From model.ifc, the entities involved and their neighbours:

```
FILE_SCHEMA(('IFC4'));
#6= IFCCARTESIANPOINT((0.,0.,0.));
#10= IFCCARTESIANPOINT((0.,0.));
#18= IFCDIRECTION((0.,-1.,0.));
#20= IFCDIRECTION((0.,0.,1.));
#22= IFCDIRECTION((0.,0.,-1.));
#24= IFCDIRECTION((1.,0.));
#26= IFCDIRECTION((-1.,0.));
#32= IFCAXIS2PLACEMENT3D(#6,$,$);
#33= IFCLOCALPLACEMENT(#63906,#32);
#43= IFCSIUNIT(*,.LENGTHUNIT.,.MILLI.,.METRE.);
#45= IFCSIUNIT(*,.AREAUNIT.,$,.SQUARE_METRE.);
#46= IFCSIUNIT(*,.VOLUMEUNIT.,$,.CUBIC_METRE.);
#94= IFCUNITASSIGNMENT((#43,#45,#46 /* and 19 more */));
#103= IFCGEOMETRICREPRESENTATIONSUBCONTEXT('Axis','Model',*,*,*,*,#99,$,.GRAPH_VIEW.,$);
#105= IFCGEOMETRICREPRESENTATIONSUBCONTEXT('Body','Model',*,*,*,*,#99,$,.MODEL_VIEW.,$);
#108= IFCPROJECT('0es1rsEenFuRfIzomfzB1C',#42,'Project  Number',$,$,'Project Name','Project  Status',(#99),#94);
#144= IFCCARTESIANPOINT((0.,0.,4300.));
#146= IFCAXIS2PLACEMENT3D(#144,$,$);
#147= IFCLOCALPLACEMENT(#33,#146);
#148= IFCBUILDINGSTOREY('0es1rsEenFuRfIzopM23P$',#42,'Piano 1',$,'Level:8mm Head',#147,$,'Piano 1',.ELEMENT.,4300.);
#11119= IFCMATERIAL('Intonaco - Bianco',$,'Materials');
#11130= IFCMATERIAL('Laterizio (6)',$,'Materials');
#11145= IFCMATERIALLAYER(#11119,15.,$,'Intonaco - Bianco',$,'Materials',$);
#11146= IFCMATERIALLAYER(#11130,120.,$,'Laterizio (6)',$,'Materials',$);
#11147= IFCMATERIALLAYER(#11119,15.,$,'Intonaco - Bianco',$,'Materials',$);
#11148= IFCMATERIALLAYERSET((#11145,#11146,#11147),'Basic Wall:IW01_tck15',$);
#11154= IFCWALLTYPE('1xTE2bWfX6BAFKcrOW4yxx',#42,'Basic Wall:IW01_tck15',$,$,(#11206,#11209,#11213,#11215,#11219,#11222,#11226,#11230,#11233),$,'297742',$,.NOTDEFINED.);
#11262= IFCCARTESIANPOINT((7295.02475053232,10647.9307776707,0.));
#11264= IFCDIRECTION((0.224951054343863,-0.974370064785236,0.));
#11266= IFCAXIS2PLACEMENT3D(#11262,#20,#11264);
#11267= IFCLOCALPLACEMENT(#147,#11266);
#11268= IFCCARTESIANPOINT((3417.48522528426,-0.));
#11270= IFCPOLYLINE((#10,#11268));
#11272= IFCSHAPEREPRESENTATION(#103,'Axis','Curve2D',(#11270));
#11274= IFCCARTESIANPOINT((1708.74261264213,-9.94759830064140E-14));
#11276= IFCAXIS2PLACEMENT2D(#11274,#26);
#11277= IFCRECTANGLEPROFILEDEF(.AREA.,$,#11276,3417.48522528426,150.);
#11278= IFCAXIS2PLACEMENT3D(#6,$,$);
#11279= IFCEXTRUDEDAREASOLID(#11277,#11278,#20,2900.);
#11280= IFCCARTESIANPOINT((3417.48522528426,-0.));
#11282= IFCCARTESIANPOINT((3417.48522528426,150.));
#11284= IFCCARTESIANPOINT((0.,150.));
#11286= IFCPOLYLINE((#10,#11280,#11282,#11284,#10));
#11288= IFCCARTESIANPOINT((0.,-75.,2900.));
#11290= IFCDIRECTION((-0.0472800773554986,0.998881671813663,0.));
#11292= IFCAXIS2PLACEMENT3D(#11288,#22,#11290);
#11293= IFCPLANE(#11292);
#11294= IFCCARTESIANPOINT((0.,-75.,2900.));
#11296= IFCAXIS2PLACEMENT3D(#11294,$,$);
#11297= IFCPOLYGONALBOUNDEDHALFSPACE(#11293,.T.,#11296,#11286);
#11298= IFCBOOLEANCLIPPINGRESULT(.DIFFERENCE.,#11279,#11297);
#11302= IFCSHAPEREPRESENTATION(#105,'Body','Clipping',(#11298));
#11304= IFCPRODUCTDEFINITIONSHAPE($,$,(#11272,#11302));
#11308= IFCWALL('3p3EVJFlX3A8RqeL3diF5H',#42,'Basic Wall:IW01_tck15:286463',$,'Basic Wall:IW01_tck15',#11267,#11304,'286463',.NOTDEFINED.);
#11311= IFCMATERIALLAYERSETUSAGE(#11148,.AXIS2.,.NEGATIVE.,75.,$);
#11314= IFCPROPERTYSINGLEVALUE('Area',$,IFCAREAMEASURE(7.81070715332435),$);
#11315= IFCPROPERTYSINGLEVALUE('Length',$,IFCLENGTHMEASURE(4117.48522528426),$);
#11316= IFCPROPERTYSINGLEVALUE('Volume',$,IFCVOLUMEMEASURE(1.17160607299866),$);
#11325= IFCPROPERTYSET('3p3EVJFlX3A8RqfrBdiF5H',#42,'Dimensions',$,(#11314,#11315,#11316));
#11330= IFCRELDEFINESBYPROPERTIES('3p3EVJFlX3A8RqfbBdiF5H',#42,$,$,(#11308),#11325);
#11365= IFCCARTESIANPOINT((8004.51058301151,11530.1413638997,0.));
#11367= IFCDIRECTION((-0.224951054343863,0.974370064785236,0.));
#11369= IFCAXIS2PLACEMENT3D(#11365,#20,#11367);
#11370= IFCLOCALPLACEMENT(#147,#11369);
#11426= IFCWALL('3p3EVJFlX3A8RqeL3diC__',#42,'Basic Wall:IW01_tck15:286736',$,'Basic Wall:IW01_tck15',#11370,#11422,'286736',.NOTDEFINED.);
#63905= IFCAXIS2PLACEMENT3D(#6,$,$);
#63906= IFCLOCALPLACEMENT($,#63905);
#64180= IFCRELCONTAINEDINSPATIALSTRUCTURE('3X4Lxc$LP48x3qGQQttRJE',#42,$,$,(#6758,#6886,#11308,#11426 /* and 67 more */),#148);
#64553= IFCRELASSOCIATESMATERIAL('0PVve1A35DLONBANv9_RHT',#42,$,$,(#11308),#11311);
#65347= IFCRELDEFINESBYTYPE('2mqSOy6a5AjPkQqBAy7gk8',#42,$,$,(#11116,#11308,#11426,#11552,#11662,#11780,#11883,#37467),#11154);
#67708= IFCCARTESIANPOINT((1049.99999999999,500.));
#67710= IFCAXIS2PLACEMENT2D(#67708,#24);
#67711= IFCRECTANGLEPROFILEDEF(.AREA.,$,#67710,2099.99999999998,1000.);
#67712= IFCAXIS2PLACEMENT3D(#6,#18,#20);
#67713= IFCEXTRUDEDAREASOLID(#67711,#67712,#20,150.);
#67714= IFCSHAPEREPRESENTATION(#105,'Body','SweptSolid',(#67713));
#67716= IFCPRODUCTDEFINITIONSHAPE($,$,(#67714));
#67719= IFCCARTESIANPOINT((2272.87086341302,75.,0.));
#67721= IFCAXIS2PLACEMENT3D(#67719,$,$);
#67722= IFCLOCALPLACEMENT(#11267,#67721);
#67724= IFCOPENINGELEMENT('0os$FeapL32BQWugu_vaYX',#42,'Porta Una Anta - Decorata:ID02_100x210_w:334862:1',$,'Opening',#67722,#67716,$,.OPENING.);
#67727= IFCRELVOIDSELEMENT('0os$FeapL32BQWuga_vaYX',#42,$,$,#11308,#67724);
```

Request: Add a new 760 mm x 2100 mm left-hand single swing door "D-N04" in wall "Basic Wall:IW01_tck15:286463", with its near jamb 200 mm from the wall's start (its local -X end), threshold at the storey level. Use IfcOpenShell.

```python
import numpy as np
import ifcopenshell
import ifcopenshell.api.feature
import ifcopenshell.api.geometry
import ifcopenshell.api.pset
import ifcopenshell.api.root
import ifcopenshell.api.spatial
import ifcopenshell.geom
import ifcopenshell.util.element
import ifcopenshell.util.placement
import ifcopenshell.util.representation
import ifcopenshell.util.shape
import ifcopenshell.util.unit

model = ifcopenshell.open("model.ifc")
unit_scale = ifcopenshell.util.unit.calculate_unit_scale(model)
area_scale = ifcopenshell.util.unit.calculate_unit_scale(model, "AREAUNIT")
volume_scale = ifcopenshell.util.unit.calculate_unit_scale(model, "VOLUMEUNIT")
settings = ifcopenshell.geom.settings()


def volume(element):
    """Net volume in cubic metres, openings subtracted."""
    shape = ifcopenshell.geom.create_shape(settings, element)
    return ifcopenshell.util.shape.get_volume(shape.geometry)


wall = model.by_id(11308)
storey = ifcopenshell.util.element.get_container(wall, ifc_class="IfcBuildingStorey")
context = ifcopenshell.util.representation.get_context(model, "Model", "Body", "MODEL_VIEW")
before = volume(wall)

width, height, from_end, sill = 0.76, 2.1, 0.2, 0.0  # metres

# The wall runs along its own X axis, and the end named is its -X end.
wall_shape = ifcopenshell.geom.create_shape(settings, wall)
x, y, z = ifcopenshell.util.shape.get_vertices(wall_shape.geometry).T
start = x.min() + from_end
face, thickness = float(y.min()), float(y.max() - y.min())
wall_matrix = ifcopenshell.util.placement.get_local_placement(wall.ObjectPlacement)
level = ifcopenshell.util.placement.get_local_placement(storey.ObjectPlacement)[2, 3]


def in_wall(x, y):
    """Placement at x, y metres in the wall's axes, at sill height."""
    matrix = wall_matrix.copy()
    matrix[:, 3] = wall_matrix @ np.array([x / unit_scale, y / unit_scale, 0.0, 1.0])
    matrix[2, 3] = level + sill / unit_scale
    return matrix


# Opening: a box that overshoots both wall faces by 50 mm.
opening = ifcopenshell.api.root.create_entity(model, ifc_class="IfcOpeningElement", predefined_type="OPENING")
box = ifcopenshell.api.geometry.add_wall_representation(
    model, context=context, length=width, height=height, thickness=thickness + 0.1
)
ifcopenshell.api.geometry.assign_representation(model, product=opening, representation=box)
ifcopenshell.api.geometry.edit_object_placement(model, product=opening, matrix=in_wall(start, face - 0.05), is_si=False)
ifcopenshell.api.feature.add_feature(model, feature=opening, element=wall)

door = ifcopenshell.api.root.create_entity(model, ifc_class="IfcDoor", name="D-N04", predefined_type="DOOR")
door.OverallWidth, door.OverallHeight = width / unit_scale, height / unit_scale
door.OperationType = "SINGLE_SWING_LEFT"
body = ifcopenshell.api.geometry.add_door_representation(
    model,
    context=context,
    overall_width=door.OverallWidth,
    overall_height=door.OverallHeight,
    operation_type="SINGLE_SWING_LEFT",
    lining_properties={"LiningDepth": thickness / unit_scale, "ThresholdDepth": thickness / unit_scale},
)
ifcopenshell.api.geometry.assign_representation(model, product=door, representation=body)
ifcopenshell.api.spatial.assign_container(model, products=[door], relating_structure=storey)
ifcopenshell.api.feature.add_filling(model, opening=opening, element=door)

# The lining spans the wall, so the door starts at the wall face.
ifcopenshell.api.geometry.edit_object_placement(model, product=door, matrix=in_wall(start, face), is_si=False)

after = volume(wall)

# Update the wall's stored quantities.
pset = model.by_id(ifcopenshell.util.element.get_pset(wall, "Dimensions", should_inherit=False)["id"])
ifcopenshell.api.pset.edit_pset(model, pset=pset, properties={
    "Area": model.create_entity("IfcAreaMeasure", after / thickness / area_scale),
    "Volume": model.create_entity("IfcVolumeMeasure", after / volume_scale),
})

print(f"wall volume {before:.3f} -> {after:.3f} m3")

model.write("model-out.ifc")
```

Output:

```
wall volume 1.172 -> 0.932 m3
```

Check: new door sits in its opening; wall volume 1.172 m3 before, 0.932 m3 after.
